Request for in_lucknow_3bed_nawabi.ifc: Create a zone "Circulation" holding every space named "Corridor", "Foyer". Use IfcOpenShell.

First a look at what the model holds.

```python
import ifcopenshell

model = ifcopenshell.open("in_lucknow_3bed_nawabi.ifc")
print(model.schema)
seen = {}
for space in model.by_type("IfcSpace"):
    seen[space.LongName] = seen.get(space.LongName, 0) + 1
for name, count in sorted(seen.items(), key=str):
    print(count, "x", name)
print("zones:", [z.Name for z in model.by_type("IfcZone")][:20])
```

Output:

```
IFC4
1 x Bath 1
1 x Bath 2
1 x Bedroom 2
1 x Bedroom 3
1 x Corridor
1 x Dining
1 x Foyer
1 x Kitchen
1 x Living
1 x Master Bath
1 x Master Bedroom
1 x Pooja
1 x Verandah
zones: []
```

```python
import ifcopenshell
import ifcopenshell.api.group
import ifcopenshell.api.root

model = ifcopenshell.open("in_lucknow_3bed_nawabi.ifc")

names = {"Corridor", "Foyer"}
spaces = [s for s in model.by_type("IfcSpace") if s.LongName in names]

zone = ifcopenshell.api.root.create_entity(model, ifc_class="IfcZone", name="Circulation")
ifcopenshell.api.group.assign_group(model, products=spaces, group=zone)
print(len(spaces), "spaces in", zone.Name)

model.write("in_lucknow_3bed_nawabi-out.ifc")
```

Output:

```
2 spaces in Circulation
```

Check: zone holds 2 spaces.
